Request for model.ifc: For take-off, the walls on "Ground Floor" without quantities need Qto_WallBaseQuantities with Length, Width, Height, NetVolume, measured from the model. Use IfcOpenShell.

First a look at what the model holds.

```python
import ifcopenshell
import ifcopenshell.util.element
import ifcopenshell.util.unit

model = ifcopenshell.open("model.ifc")
print(model.schema)
for unit_type in ("LENGTHUNIT", "AREAUNIT", "VOLUMEUNIT"):
    print(unit_type, ifcopenshell.util.unit.calculate_unit_scale(model, unit_type))
storey = next(s for s in model.by_type("IfcBuildingStorey") if s.Name == "Ground Floor")
walls = [e for e in ifcopenshell.util.element.get_decomposition(storey) if e.is_a("IfcWall")]
for e in sorted(walls, key=lambda e: e.id()):
    print(e.id(), e.is_a(), e.Name, list(ifcopenshell.util.element.get_psets(e, qtos_only=True)), sep=" | ")
```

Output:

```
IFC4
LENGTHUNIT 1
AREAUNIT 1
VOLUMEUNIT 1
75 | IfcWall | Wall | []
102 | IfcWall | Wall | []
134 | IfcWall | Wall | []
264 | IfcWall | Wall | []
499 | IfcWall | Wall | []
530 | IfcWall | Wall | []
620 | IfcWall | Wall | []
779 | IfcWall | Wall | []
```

```python
import ifcopenshell
import ifcopenshell.api.pset
import ifcopenshell.geom
import ifcopenshell.util.element
import ifcopenshell.util.shape
import ifcopenshell.util.unit

model = ifcopenshell.open("model.ifc")
unit_scale = ifcopenshell.util.unit.calculate_unit_scale(model)
volume_scale = ifcopenshell.util.unit.calculate_unit_scale(model, "VOLUMEUNIT")
settings = ifcopenshell.geom.settings()

storey = next(s for s in model.by_type("IfcBuildingStorey") if s.Name == "Ground Floor")
walls = [e for e in ifcopenshell.util.element.get_decomposition(storey) if e.is_a("IfcWall")]

for e in sorted(walls, key=lambda e: e.id()):
    if ifcopenshell.util.element.get_psets(e, qtos_only=True, should_inherit=False):
        continue
    # Geometry comes back in metres, in the element's own axes.
    shape = ifcopenshell.geom.create_shape(settings, e)
    values = {
        "Length": ifcopenshell.util.shape.get_x(shape.geometry) / unit_scale,
        "Width": ifcopenshell.util.shape.get_y(shape.geometry) / unit_scale,
        "Height": ifcopenshell.util.shape.get_z(shape.geometry) / unit_scale,
        "NetVolume": ifcopenshell.util.shape.get_volume(shape.geometry) / volume_scale,
    }
    qto = ifcopenshell.api.pset.add_qto(model, product=e, name="Qto_WallBaseQuantities")
    ifcopenshell.api.pset.edit_qto(model, qto=qto, properties=values)
    print(e.id(), {k: round(v, 3) for k, v in values.items()})

model.write("model_edited.ifc")
```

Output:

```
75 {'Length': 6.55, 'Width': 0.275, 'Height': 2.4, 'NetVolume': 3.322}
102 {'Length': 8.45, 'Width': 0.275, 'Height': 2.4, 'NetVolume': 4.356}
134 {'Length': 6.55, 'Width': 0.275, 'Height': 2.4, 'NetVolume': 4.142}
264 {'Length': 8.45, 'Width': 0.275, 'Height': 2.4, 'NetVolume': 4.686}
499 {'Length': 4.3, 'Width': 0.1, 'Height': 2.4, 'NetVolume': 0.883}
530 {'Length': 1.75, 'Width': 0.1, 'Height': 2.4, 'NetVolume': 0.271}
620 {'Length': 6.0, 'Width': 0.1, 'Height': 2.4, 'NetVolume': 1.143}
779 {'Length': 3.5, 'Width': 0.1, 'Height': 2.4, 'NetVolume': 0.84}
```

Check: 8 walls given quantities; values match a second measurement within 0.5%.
